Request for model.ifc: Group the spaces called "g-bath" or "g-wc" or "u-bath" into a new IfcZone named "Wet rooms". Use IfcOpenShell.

First a look at what the model holds.

```python
import ifcopenshell

model = ifcopenshell.open("model.ifc")
print(model.schema)
seen = {}
for space in model.by_type("IfcSpace"):
    seen[space.LongName] = seen.get(space.LongName, 0) + 1
for name, count in sorted(seen.items(), key=str):
    print(count, "x", name)
print("zones:", [z.Name for z in model.by_type("IfcZone")][:20])
```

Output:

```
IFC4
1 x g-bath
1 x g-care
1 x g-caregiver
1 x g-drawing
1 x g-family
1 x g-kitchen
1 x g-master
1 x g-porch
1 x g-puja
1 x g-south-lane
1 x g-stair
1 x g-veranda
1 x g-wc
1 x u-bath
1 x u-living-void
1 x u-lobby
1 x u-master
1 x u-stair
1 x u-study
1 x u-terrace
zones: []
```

```python
import ifcopenshell
import ifcopenshell.api.group
import ifcopenshell.api.root

model = ifcopenshell.open("model.ifc")

names = {"g-bath", "g-wc", "u-bath"}
spaces = [s for s in model.by_type("IfcSpace") if s.LongName in names]

zone = ifcopenshell.api.root.create_entity(model, ifc_class="IfcZone", name="Wet rooms")
ifcopenshell.api.group.assign_group(model, products=spaces, group=zone)
print(len(spaces), "spaces in", zone.Name)

model.write("model_updated.ifc")
```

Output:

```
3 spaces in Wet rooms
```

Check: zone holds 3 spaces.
